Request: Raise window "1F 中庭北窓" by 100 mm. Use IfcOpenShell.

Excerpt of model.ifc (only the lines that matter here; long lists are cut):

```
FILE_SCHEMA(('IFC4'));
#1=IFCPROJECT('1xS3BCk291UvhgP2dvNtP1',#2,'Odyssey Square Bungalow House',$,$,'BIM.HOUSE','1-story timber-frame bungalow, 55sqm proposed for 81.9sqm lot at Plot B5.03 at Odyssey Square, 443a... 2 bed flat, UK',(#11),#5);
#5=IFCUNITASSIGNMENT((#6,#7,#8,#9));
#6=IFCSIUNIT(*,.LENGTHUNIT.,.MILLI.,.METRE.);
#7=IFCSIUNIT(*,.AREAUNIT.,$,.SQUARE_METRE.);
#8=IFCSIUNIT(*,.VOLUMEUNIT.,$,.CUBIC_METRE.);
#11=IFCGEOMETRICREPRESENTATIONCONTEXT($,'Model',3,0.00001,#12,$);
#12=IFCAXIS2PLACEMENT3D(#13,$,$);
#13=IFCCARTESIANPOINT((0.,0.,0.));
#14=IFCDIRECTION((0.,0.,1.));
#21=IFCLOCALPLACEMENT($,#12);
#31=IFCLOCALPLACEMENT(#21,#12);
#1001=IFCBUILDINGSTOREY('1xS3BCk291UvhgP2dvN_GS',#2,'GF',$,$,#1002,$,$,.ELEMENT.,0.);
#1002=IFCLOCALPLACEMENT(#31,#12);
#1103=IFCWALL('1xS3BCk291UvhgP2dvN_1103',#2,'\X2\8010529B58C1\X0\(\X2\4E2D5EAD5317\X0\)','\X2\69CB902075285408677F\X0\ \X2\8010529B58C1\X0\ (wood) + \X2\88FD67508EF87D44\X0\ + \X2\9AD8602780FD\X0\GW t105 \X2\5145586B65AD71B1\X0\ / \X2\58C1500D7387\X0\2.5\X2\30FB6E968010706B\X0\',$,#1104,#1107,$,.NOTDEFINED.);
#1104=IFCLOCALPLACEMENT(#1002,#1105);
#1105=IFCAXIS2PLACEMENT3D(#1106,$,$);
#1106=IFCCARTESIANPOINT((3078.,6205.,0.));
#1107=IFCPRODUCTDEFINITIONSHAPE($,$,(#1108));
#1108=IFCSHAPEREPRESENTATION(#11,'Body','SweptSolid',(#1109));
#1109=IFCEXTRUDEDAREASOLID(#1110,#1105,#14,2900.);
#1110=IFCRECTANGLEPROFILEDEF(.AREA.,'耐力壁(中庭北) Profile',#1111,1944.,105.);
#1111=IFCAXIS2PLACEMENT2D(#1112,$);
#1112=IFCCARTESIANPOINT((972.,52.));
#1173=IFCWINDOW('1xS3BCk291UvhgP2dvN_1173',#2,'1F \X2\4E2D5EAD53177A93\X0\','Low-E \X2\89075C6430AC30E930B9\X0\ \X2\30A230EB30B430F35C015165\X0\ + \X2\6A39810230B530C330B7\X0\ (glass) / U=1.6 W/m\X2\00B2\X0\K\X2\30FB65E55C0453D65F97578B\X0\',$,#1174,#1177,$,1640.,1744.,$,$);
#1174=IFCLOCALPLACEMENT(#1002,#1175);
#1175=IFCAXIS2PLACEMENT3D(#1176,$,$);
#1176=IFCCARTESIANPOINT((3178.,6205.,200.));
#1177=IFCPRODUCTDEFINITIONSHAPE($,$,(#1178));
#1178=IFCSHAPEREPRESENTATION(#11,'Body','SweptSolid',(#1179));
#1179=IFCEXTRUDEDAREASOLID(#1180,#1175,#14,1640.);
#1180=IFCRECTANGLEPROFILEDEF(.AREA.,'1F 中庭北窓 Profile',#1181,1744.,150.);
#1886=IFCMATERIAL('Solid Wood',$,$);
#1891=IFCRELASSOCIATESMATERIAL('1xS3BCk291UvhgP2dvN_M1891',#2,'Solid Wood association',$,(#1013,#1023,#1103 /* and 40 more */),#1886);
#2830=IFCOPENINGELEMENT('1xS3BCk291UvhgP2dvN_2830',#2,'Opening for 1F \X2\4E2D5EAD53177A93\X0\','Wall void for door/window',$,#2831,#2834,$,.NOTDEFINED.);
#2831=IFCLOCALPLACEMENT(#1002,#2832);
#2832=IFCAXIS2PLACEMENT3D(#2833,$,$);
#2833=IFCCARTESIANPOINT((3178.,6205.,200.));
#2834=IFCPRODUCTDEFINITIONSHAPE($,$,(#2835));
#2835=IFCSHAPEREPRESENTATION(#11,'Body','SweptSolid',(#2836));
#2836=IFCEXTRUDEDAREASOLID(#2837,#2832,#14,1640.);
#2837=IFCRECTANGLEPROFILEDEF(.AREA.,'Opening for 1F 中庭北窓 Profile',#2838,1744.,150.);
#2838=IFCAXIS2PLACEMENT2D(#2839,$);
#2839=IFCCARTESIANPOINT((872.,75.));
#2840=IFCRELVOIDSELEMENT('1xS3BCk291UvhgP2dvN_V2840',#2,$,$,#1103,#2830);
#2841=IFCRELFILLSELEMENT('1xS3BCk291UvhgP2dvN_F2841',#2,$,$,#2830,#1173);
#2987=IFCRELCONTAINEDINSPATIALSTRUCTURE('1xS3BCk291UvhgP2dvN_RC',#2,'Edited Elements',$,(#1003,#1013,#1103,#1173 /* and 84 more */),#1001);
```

```python
import numpy as np
import ifcopenshell
import ifcopenshell.api.geometry
import ifcopenshell.util.placement
import ifcopenshell.util.unit

model = ifcopenshell.open("model.ifc")
unit_scale = ifcopenshell.util.unit.calculate_unit_scale(model)

window = model.by_guid("1xS3BCk291UvhgP2dvN_1173")
opening = window.FillsVoids[0].RelatingOpeningElement
dz = 0.1 / unit_scale

shift = np.array([0.0, 0.0, dz])
# The window is not placed relative to its opening, so move both.
for product in (opening, window):
    matrix = ifcopenshell.util.placement.get_local_placement(product.ObjectPlacement)
    matrix[:3, 3] += shift
    ifcopenshell.api.geometry.edit_object_placement(model, product=product, matrix=matrix, is_si=False)

print(f"moved by {dz * unit_scale:+.3f} m")

model.write("model_edited.ifc")
```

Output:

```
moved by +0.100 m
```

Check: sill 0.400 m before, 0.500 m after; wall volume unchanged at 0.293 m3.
